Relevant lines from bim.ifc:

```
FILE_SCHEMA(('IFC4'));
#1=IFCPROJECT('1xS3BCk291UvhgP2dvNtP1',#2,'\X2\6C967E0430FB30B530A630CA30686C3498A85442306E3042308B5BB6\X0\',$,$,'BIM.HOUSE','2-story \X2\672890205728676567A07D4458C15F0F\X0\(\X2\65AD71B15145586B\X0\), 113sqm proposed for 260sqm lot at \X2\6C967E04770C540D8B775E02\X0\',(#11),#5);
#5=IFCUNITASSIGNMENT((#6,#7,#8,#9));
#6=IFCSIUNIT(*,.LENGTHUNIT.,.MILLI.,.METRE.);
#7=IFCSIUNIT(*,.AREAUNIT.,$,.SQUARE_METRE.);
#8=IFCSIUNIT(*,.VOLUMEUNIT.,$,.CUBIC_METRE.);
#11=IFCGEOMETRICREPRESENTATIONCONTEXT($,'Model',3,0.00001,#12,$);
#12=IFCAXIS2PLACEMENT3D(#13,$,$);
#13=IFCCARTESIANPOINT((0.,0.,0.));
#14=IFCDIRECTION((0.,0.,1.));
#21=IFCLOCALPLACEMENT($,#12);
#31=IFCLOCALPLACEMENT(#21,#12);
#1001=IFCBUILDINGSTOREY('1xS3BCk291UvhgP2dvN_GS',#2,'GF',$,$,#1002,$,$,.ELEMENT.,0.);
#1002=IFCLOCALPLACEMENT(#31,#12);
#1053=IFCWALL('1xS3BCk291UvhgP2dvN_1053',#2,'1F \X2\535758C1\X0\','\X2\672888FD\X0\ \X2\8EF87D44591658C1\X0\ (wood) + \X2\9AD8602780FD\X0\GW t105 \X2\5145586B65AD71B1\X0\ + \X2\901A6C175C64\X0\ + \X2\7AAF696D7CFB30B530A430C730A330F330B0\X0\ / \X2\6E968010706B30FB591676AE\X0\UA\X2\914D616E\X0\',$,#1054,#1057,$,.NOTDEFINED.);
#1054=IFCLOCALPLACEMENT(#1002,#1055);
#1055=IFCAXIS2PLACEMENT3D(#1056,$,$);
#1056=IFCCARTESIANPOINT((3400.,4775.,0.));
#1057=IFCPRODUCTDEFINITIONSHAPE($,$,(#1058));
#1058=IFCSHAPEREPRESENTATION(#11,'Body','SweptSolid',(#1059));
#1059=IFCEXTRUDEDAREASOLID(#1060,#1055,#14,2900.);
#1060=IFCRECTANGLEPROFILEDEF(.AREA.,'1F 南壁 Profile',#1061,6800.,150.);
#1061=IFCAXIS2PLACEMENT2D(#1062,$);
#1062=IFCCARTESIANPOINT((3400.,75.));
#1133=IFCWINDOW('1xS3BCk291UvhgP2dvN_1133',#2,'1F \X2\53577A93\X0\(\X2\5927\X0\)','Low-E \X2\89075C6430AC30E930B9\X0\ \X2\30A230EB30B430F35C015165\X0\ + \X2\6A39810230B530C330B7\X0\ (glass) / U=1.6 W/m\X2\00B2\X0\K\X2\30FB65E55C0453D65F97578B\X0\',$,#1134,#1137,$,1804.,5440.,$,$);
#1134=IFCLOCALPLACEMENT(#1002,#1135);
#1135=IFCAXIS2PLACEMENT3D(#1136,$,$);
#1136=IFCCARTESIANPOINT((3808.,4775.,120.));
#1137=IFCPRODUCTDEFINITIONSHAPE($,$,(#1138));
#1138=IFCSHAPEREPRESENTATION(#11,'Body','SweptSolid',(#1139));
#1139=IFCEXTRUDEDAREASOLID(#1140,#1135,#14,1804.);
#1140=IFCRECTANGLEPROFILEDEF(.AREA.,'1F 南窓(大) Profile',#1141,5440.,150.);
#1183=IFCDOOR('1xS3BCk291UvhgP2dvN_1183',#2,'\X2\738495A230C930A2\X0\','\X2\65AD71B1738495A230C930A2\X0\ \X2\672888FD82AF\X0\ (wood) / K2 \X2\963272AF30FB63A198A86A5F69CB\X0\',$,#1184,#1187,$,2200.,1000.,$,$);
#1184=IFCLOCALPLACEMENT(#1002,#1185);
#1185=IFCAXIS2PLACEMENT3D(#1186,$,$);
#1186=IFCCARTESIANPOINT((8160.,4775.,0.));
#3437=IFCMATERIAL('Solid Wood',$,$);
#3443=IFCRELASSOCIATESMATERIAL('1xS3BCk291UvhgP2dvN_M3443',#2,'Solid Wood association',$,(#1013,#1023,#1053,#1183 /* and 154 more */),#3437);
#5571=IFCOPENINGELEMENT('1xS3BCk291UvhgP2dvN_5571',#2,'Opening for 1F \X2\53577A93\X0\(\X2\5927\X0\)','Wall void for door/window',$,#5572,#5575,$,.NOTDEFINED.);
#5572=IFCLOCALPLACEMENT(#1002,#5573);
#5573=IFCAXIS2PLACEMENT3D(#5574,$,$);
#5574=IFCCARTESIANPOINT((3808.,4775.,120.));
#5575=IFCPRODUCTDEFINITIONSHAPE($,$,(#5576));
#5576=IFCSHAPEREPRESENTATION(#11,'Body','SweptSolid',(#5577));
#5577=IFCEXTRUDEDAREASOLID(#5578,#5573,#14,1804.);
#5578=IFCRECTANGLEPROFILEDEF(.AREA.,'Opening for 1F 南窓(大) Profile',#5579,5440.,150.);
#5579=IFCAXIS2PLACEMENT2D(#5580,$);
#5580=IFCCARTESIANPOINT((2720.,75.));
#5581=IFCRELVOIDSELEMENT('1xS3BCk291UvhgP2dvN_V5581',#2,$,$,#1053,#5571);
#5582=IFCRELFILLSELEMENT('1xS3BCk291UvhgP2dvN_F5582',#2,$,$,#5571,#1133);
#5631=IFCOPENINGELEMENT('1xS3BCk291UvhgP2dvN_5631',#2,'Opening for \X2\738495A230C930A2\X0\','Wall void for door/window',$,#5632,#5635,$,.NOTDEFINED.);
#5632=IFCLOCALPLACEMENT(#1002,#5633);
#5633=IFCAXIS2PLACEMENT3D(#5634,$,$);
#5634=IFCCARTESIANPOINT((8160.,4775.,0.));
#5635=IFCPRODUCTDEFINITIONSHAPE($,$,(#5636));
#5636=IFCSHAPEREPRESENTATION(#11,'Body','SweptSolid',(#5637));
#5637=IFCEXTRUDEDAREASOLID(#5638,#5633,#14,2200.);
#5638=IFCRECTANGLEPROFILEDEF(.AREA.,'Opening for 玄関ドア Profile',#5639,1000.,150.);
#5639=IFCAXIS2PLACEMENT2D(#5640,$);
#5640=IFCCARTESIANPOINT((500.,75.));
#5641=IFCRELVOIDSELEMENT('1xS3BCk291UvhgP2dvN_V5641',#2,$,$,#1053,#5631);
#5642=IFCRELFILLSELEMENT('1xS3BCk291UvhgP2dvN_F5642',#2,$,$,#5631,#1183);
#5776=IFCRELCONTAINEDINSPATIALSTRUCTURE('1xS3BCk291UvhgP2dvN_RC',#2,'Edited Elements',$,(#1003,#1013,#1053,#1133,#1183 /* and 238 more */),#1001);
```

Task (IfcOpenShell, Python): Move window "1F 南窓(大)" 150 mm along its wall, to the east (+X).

```python
import ifcopenshell
import ifcopenshell.api.geometry
import ifcopenshell.util.placement

model = ifcopenshell.open("bim.ifc")

window = model.by_guid("1xS3BCk291UvhgP2dvN_1133")
opening = window.FillsVoids[0].RelatingOpeningElement
wall = opening.VoidsElements[0].RelatingBuildingElement

wall_matrix = ifcopenshell.util.placement.get_local_placement(wall.ObjectPlacement)
shift = wall_matrix[:3, 0] * 150.0
before = ifcopenshell.util.placement.get_local_placement(window.ObjectPlacement)[:3, 3].copy()

# The window is not placed relative to its opening, so move both.
for product in (opening, window):
    matrix = ifcopenshell.util.placement.get_local_placement(product.ObjectPlacement)
    matrix[:3, 3] += shift
    ifcopenshell.api.geometry.edit_object_placement(model, product=product, matrix=matrix, is_si=False)

after = ifcopenshell.util.placement.get_local_placement(window.ObjectPlacement)[:3, 3]
print("window moved by", (after - before).round(3) + 0.0)

model.write("bim_rev.ifc")
```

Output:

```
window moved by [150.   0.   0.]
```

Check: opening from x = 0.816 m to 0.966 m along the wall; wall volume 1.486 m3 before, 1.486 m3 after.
